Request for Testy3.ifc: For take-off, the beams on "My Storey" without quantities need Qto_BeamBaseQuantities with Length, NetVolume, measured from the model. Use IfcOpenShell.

First a look at what the model holds.

```python
import ifcopenshell
import ifcopenshell.util.element
import ifcopenshell.util.unit

model = ifcopenshell.open("Testy3.ifc")
print(model.schema)
for unit_type in ("LENGTHUNIT", "AREAUNIT", "VOLUMEUNIT"):
    print(unit_type, ifcopenshell.util.unit.calculate_unit_scale(model, unit_type))
storey = next(s for s in model.by_type("IfcBuildingStorey") if s.Name == "My Storey")
beams = [e for e in ifcopenshell.util.element.get_decomposition(storey) if e.is_a("IfcBeam")]
for e in sorted(beams, key=lambda e: e.id()):
    print(e.id(), e.is_a(), e.Name, list(ifcopenshell.util.element.get_psets(e, qtos_only=True)), sep=" | ")
```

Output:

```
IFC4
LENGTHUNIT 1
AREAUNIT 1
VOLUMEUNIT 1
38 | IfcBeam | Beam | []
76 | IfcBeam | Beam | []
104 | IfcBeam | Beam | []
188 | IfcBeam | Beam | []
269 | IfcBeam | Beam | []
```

```python
import ifcopenshell
import ifcopenshell.api.pset
import ifcopenshell.geom
import ifcopenshell.util.element
import ifcopenshell.util.shape
import ifcopenshell.util.unit

model = ifcopenshell.open("Testy3.ifc")
unit_scale = ifcopenshell.util.unit.calculate_unit_scale(model)
volume_scale = ifcopenshell.util.unit.calculate_unit_scale(model, "VOLUMEUNIT")
settings = ifcopenshell.geom.settings()

storey = next(s for s in model.by_type("IfcBuildingStorey") if s.Name == "My Storey")
beams = [e for e in ifcopenshell.util.element.get_decomposition(storey) if e.is_a("IfcBeam")]

for e in sorted(beams, key=lambda e: e.id()):
    if ifcopenshell.util.element.get_psets(e, qtos_only=True, should_inherit=False):
        continue
    # Geometry comes back in metres, in the element's own axes.
    shape = ifcopenshell.geom.create_shape(settings, e)
    values = {
        "Length": ifcopenshell.util.shape.get_max_xyz(shape.geometry) / unit_scale,
        "NetVolume": ifcopenshell.util.shape.get_volume(shape.geometry) / volume_scale,
    }
    qto = ifcopenshell.api.pset.add_qto(model, product=e, name="Qto_BeamBaseQuantities")
    ifcopenshell.api.pset.edit_qto(model, qto=qto, properties=values)
    print(e.id(), {k: round(v, 3) for k, v in values.items()})

model.write("Testy3_v2.ifc")
```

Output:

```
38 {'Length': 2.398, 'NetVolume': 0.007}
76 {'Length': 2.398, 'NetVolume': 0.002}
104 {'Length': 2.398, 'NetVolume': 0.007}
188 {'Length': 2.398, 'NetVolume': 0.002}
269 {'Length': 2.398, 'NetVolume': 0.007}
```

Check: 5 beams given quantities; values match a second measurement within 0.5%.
